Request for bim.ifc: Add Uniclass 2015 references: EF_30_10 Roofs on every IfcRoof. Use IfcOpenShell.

First a look at what the model holds.

```python
import ifcopenshell

model = ifcopenshell.open("bim.ifc")
print(model.schema)
print("classifications:", [c.Name for c in model.by_type("IfcClassification")])
for ifc_class in ("IfcDoor", "IfcRoof", "IfcStair", "IfcWall", "IfcWindow"):
    print(ifc_class, len(model.by_type(ifc_class)))
```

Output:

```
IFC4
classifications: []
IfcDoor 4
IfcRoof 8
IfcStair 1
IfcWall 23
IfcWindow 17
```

```python
import ifcopenshell
import ifcopenshell.api.classification

model = ifcopenshell.open("bim.ifc")

system = ifcopenshell.api.classification.add_classification(model, classification="Uniclass 2015")

codes = {
    "IfcRoof": ("EF_30_10", "Roofs"),
}
for ifc_class, (code, name) in codes.items():
    products = model.by_type(ifc_class)
    ifcopenshell.api.classification.add_reference(
        model, products=products, classification=system, identification=code, name=name
    )
    print(code, len(products))

model.write("bim_edited.ifc")
```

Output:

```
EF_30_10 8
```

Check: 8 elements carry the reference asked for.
